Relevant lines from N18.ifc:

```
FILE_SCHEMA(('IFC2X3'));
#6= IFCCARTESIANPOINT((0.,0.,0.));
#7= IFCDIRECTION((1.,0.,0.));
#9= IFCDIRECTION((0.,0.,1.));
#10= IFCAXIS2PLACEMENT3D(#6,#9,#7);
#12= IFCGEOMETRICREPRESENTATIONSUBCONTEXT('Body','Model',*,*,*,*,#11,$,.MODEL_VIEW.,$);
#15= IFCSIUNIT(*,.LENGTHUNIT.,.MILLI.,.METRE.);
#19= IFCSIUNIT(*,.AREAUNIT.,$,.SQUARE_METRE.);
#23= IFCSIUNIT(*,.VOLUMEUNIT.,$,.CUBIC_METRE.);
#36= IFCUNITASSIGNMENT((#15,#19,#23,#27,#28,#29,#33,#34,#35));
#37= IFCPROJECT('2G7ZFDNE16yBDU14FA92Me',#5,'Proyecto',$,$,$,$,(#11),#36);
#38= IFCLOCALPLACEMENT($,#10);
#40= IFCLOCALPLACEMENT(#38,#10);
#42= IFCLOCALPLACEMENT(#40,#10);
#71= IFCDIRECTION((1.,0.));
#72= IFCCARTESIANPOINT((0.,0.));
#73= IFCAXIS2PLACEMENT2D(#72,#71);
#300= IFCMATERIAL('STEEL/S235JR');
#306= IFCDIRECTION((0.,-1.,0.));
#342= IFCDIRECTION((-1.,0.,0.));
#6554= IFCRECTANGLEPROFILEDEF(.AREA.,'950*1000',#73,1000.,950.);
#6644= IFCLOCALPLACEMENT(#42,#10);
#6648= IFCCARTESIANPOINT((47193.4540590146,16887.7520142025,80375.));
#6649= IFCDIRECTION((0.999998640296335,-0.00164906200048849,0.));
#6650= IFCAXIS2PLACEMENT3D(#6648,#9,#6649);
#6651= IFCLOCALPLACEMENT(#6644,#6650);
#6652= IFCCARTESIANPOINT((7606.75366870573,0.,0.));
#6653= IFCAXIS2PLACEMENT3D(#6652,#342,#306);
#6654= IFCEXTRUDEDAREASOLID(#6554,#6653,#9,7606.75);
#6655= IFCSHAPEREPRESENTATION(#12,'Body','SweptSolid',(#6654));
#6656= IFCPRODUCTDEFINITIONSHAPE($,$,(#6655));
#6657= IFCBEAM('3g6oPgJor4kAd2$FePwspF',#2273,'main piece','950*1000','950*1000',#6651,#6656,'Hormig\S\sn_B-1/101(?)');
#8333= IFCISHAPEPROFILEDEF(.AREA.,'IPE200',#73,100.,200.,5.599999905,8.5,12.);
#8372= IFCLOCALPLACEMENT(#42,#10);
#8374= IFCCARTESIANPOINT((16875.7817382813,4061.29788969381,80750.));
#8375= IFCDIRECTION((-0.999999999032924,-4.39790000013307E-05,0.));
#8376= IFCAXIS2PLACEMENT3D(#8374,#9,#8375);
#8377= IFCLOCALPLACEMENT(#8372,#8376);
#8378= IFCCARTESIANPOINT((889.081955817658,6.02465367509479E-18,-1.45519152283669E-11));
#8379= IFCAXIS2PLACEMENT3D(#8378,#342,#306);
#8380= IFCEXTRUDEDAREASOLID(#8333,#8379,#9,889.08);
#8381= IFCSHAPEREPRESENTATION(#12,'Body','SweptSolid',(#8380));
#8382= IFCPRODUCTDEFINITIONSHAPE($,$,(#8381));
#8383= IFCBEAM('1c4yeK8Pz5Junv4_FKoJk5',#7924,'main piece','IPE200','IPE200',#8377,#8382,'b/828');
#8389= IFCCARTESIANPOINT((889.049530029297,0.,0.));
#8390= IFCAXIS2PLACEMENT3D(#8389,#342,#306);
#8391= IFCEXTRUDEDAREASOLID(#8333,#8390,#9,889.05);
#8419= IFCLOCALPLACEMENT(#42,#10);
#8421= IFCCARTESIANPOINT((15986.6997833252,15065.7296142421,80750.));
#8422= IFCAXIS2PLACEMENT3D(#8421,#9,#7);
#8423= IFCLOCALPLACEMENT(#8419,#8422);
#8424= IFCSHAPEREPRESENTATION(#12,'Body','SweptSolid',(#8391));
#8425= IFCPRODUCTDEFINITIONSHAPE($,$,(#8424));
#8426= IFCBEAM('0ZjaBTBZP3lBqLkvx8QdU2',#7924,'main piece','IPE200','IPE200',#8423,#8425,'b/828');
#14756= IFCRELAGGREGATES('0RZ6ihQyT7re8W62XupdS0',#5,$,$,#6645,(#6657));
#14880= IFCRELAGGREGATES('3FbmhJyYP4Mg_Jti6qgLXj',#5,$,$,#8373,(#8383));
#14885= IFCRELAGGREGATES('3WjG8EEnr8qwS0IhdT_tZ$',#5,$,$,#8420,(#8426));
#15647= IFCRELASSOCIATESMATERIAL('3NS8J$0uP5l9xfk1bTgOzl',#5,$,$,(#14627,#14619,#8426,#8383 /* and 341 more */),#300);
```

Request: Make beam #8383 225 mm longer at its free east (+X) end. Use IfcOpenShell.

```python
import ifcopenshell
import ifcopenshell.util.representation
import ifcopenshell.util.unit

model = ifcopenshell.open("N18.ifc")
unit_scale = ifcopenshell.util.unit.calculate_unit_scale(model)

member = model.by_id(8383)
change = 0.225 / unit_scale

# The extrusion runs towards the end named, so only its depth changes.
body = ifcopenshell.util.representation.get_representation(member, "Model", "Body")
solid = body.Items[0]
old_length = solid.Depth
solid.Depth += change

print(f"length {old_length:g} -> {solid.Depth:g}")

model.write("N18_rev.ifc")
```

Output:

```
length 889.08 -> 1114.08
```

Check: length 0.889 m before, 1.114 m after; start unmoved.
